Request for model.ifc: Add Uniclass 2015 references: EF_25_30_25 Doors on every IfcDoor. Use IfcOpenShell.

First a look at what the model holds.

```python
import ifcopenshell

model = ifcopenshell.open("model.ifc")
print(model.schema)
print("classifications:", [c.Name for c in model.by_type("IfcClassification")])
for ifc_class in ("IfcDoor", "IfcRoof", "IfcStair", "IfcWall", "IfcWindow"):
    print(ifc_class, len(model.by_type(ifc_class)))
```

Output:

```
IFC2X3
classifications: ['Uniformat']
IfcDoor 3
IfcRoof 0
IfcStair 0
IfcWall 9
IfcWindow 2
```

```python
import ifcopenshell
import ifcopenshell.api.classification

model = ifcopenshell.open("model.ifc")

# IFC2X3 requires Source and Edition and has no link from the project to the system.
system = model.create_entity("IfcClassification", Source="NBS", Edition="2015", Name="Uniclass 2015")

codes = {
    "IfcDoor": ("EF_25_30_25", "Doors"),
}
for ifc_class, (code, name) in codes.items():
    products = model.by_type(ifc_class)
    ifcopenshell.api.classification.add_reference(
        model, products=products, classification=system, identification=code, name=name
    )
    print(code, len(products))

model.write("model_edited.ifc")
```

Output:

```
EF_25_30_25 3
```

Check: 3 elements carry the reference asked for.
